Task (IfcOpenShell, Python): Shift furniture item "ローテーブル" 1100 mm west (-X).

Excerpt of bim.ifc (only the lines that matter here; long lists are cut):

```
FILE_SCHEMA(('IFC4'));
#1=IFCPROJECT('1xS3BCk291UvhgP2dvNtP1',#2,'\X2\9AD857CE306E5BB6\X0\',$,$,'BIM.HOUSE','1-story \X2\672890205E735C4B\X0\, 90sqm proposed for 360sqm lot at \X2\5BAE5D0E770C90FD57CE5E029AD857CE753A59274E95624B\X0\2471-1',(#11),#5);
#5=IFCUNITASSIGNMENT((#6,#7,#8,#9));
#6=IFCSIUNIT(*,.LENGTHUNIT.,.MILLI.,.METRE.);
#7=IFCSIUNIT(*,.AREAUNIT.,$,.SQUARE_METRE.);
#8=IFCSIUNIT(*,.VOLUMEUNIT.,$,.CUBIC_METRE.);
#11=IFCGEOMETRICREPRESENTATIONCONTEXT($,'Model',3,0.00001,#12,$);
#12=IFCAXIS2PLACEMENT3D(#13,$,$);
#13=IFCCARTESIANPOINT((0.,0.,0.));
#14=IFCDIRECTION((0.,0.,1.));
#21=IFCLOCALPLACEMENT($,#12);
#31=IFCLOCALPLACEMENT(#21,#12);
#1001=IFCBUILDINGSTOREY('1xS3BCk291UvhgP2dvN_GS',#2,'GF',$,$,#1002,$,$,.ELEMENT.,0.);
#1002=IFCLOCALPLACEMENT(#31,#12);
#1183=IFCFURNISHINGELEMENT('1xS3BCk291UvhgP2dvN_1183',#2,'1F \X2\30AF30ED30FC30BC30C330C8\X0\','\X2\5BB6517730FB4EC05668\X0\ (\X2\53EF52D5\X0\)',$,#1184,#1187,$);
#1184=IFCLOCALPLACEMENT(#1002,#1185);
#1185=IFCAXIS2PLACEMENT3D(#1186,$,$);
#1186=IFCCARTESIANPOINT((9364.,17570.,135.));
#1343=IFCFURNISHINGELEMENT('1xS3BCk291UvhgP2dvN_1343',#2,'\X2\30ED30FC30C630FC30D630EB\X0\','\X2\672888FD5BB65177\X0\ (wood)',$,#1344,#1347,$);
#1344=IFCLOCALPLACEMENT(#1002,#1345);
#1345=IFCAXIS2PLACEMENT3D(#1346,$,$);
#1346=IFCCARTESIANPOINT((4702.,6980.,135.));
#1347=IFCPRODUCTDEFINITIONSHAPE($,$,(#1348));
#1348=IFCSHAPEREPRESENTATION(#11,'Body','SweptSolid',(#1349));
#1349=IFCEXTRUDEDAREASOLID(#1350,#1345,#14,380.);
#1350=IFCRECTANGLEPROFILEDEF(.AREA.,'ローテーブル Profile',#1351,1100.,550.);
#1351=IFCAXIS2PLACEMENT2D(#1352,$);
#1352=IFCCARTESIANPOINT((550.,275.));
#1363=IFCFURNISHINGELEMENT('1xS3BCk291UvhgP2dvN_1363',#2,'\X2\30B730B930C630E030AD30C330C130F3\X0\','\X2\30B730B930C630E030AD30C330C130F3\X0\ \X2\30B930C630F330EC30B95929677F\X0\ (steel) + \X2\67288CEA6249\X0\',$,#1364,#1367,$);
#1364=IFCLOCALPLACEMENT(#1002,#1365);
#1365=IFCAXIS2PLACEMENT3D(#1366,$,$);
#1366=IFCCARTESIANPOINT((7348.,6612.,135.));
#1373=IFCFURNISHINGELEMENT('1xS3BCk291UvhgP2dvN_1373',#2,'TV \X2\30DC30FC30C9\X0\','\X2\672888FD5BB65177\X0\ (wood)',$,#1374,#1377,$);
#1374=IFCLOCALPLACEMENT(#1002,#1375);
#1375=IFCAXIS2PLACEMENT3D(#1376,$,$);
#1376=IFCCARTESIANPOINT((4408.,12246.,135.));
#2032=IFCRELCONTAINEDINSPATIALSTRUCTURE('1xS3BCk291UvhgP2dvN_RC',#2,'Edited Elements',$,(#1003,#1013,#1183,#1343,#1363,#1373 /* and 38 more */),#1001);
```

```python
import ifcopenshell
import ifcopenshell.api.geometry
import ifcopenshell.util.placement
import ifcopenshell.util.unit

model = ifcopenshell.open("bim.ifc")
unit_scale = ifcopenshell.util.unit.calculate_unit_scale(model)

item = model.by_id(1343)
matrix = ifcopenshell.util.placement.get_local_placement(item.ObjectPlacement)
matrix[0, 3] -= 1.1 / unit_scale
ifcopenshell.api.geometry.edit_object_placement(model, product=item, matrix=matrix, is_si=False)

print(ifcopenshell.util.placement.get_local_placement(item.ObjectPlacement).round(3) + 0.0)

model.write("bim_rev.ifc")
```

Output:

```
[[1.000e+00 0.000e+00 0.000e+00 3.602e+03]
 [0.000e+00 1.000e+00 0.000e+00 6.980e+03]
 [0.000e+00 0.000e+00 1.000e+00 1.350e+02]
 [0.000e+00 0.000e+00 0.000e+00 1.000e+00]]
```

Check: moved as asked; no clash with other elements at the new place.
